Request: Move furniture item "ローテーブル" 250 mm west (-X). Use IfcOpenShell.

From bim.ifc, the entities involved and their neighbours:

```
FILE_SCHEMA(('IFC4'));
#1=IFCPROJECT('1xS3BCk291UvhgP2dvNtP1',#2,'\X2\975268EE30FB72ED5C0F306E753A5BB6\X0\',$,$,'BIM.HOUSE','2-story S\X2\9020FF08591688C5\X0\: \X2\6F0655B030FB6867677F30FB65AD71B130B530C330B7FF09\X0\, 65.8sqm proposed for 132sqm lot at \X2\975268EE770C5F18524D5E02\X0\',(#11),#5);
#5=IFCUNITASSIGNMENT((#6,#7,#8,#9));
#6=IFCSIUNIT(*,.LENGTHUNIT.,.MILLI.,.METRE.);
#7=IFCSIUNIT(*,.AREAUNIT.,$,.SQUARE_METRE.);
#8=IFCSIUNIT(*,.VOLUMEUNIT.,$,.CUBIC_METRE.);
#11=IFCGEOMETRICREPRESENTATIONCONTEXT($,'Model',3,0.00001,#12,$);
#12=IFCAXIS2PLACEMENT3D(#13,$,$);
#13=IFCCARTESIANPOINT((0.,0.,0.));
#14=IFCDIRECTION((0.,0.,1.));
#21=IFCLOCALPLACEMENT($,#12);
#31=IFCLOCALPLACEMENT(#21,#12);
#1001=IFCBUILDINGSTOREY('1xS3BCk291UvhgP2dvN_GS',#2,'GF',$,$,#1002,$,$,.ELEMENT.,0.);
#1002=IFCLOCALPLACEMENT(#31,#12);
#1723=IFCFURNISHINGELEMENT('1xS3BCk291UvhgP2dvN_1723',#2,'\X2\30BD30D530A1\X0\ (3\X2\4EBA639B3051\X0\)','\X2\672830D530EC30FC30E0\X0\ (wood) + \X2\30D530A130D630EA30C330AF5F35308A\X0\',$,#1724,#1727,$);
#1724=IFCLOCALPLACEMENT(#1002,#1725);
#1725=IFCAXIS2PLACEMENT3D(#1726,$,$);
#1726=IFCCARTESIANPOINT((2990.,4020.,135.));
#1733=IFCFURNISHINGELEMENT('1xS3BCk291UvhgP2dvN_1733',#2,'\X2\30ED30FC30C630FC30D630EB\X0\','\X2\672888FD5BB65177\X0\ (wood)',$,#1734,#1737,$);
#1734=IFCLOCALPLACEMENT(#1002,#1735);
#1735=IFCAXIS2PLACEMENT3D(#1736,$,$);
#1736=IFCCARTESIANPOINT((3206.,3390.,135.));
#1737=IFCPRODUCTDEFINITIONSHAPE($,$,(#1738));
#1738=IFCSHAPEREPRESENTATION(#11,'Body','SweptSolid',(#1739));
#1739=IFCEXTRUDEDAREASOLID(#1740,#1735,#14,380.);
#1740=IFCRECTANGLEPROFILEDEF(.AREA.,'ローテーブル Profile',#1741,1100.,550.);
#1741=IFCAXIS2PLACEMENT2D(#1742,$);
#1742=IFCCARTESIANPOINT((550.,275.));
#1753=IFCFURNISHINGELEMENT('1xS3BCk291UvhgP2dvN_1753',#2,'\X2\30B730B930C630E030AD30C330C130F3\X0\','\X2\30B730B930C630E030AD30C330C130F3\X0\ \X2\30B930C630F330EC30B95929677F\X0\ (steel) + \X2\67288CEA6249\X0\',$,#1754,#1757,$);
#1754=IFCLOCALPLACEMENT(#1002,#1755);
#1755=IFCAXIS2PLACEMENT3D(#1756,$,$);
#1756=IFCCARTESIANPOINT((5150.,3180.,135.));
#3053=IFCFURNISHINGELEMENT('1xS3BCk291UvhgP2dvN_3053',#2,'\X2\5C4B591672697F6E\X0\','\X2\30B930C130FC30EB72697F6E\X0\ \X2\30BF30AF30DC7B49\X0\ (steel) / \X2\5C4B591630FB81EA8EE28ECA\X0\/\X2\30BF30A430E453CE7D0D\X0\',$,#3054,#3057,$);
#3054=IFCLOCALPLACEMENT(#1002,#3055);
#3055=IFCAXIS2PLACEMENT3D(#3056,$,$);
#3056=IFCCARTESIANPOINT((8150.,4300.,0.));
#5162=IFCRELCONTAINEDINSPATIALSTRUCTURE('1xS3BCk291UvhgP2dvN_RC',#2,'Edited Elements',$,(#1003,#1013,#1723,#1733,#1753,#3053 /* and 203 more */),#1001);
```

```python
import ifcopenshell
import ifcopenshell.api.geometry
import ifcopenshell.util.placement
import ifcopenshell.util.unit

model = ifcopenshell.open("bim.ifc")
unit_scale = ifcopenshell.util.unit.calculate_unit_scale(model)

item = model.by_guid("1xS3BCk291UvhgP2dvN_1733")
matrix = ifcopenshell.util.placement.get_local_placement(item.ObjectPlacement)
matrix[0, 3] -= 0.25 / unit_scale
ifcopenshell.api.geometry.edit_object_placement(model, product=item, matrix=matrix, is_si=False)

print(ifcopenshell.util.placement.get_local_placement(item.ObjectPlacement).round(3) + 0.0)

model.write("bim_updated.ifc")
```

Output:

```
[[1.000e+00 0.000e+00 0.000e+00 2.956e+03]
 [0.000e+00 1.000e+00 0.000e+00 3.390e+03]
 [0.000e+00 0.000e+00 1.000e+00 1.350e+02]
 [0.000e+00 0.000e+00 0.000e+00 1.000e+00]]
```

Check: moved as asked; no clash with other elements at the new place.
